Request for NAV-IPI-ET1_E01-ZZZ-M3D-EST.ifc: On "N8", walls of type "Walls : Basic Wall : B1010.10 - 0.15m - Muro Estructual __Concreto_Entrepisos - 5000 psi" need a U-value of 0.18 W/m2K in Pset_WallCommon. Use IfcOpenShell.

First a look at what the model holds.

```python
import ifcopenshell
import ifcopenshell.util.element

model = ifcopenshell.open("NAV-IPI-ET1_E01-ZZZ-M3D-EST.ifc")
print(model.schema)
storey = next(s for s in model.by_type("IfcBuildingStorey") if s.Name == "N8")
walls = [e for e in ifcopenshell.util.element.get_decomposition(storey) if e.is_a("IfcWall")]
seen = {}
for e in walls:
    element_type = ifcopenshell.util.element.get_type(e)
    key = (element_type.Name if element_type != e and element_type else None, ifcopenshell.util.element.get_pset(e, "Pset_WallCommon", "ThermalTransmittance"))
    seen[key] = seen.get(key, 0) + 1
for (name, value), count in sorted(seen.items(), key=str):
    print(count, "x", name, "|", value)
```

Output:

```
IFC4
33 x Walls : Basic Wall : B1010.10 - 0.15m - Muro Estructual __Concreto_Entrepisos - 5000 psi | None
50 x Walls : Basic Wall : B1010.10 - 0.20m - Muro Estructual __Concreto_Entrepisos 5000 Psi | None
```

```python
import ifcopenshell
import ifcopenshell.api.pset
import ifcopenshell.util.element

model = ifcopenshell.open("NAV-IPI-ET1_E01-ZZZ-M3D-EST.ifc")

storey = next(s for s in model.by_type("IfcBuildingStorey") if s.Name == "N8")
walls = [e for e in ifcopenshell.util.element.get_decomposition(storey) if e.is_a("IfcWall")]

count = 0
for e in walls:
    element_type = ifcopenshell.util.element.get_type(e)
    if element_type in (None, e) or element_type.Name != "Walls : Basic Wall : B1010.10 - 0.15m - Muro Estructual __Concreto_Entrepisos - 5000 psi":
        continue
    # add_pset returns the element's existing set when there is one.
    pset = ifcopenshell.api.pset.add_pset(model, product=e, name="Pset_WallCommon")
    ifcopenshell.api.pset.edit_pset(model, pset=pset, properties={"ThermalTransmittance": 0.18})
    count += 1

print(count, "walls updated")

model.write("NAV-IPI-ET1_E01-ZZZ-M3D-EST_edited.ifc")
```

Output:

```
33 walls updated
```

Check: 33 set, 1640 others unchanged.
